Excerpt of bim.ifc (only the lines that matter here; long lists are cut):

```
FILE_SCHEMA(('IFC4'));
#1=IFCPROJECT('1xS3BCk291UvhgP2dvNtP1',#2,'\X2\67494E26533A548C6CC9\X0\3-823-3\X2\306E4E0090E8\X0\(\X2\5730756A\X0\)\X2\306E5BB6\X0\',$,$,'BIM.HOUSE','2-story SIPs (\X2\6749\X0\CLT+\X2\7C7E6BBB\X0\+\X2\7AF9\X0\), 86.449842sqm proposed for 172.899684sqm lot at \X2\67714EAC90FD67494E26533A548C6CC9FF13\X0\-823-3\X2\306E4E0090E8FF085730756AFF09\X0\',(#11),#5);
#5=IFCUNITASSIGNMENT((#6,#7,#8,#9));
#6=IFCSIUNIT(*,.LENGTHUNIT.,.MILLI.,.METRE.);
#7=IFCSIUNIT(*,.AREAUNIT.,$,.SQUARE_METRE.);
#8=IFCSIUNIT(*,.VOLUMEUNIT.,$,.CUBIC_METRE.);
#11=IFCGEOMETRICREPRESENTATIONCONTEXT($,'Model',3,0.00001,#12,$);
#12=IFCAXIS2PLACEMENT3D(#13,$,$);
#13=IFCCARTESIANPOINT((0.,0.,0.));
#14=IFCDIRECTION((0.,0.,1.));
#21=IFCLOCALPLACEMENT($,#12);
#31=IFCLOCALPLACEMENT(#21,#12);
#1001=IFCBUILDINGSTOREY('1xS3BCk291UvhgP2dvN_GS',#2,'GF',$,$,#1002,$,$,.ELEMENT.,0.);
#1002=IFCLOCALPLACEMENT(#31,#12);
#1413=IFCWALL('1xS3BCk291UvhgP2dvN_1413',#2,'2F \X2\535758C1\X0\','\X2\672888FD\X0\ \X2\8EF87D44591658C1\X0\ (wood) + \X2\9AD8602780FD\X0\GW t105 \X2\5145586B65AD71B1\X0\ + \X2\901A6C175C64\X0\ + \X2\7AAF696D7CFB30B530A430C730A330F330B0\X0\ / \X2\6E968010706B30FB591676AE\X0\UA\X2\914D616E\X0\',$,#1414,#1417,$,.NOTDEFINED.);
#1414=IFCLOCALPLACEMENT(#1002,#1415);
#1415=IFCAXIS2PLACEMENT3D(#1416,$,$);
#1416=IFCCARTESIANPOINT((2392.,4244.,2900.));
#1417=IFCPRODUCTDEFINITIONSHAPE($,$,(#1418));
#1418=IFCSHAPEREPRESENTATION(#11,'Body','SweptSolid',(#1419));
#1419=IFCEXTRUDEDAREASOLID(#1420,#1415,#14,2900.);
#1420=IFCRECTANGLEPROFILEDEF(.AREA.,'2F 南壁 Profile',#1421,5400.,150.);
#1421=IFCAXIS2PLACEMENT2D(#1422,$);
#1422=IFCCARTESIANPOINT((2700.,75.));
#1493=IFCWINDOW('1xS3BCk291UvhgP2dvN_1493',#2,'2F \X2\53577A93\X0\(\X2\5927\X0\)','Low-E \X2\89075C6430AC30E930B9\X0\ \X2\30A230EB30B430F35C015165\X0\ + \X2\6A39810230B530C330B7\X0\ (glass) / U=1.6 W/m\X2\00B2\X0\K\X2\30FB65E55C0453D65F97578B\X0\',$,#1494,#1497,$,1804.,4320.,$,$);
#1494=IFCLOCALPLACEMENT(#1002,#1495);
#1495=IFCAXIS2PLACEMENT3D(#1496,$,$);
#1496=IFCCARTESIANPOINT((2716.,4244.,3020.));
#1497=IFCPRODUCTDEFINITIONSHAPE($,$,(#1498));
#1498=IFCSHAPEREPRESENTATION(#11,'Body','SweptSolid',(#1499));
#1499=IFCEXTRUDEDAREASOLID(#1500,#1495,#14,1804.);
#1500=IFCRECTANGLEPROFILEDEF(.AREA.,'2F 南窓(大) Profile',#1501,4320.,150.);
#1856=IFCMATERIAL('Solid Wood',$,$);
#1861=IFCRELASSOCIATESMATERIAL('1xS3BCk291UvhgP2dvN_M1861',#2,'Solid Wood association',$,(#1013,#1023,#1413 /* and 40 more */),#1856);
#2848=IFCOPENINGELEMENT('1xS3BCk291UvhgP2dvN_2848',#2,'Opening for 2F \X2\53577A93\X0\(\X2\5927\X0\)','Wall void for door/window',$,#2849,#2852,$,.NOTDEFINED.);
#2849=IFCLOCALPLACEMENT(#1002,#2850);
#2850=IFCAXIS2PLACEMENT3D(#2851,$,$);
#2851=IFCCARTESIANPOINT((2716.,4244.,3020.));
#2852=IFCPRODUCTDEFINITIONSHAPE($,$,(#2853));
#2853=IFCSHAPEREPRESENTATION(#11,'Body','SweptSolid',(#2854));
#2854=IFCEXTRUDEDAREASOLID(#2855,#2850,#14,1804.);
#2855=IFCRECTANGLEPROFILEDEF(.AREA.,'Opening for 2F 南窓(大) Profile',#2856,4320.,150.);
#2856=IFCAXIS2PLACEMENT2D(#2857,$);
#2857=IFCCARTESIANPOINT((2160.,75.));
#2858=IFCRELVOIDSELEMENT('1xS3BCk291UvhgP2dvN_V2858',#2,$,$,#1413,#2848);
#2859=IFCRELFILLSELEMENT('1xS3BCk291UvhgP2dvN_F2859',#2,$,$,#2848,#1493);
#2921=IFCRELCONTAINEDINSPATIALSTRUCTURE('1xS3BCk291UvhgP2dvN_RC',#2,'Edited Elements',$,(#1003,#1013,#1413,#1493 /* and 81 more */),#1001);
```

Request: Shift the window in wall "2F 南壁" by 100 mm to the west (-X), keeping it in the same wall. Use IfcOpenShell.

```python
import ifcopenshell
import ifcopenshell.api.geometry
import ifcopenshell.util.placement
import ifcopenshell.util.unit

model = ifcopenshell.open("bim.ifc")
unit_scale = ifcopenshell.util.unit.calculate_unit_scale(model)

window = model.by_guid("1xS3BCk291UvhgP2dvN_1493")
opening = window.FillsVoids[0].RelatingOpeningElement
wall = opening.VoidsElements[0].RelatingBuildingElement

wall_matrix = ifcopenshell.util.placement.get_local_placement(wall.ObjectPlacement)
shift = wall_matrix[:3, 0] * -0.1 / unit_scale
before = ifcopenshell.util.placement.get_local_placement(window.ObjectPlacement)[:3, 3].copy()

# The window is not placed relative to its opening, so move both.
for product in (opening, window):
    matrix = ifcopenshell.util.placement.get_local_placement(product.ObjectPlacement)
    matrix[:3, 3] += shift
    ifcopenshell.api.geometry.edit_object_placement(model, product=product, matrix=matrix, is_si=False)

after = ifcopenshell.util.placement.get_local_placement(window.ObjectPlacement)[:3, 3]
print("window moved by", (after - before).round(3) + 0.0)

model.write("bim_updated.ifc")
```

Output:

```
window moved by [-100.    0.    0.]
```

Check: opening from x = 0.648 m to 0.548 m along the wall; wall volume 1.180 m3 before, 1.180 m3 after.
